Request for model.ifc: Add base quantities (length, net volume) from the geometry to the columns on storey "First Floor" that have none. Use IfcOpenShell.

First a look at what the model holds.

```python
import ifcopenshell
import ifcopenshell.util.element
import ifcopenshell.util.unit

model = ifcopenshell.open("model.ifc")
print(model.schema)
for unit_type in ("LENGTHUNIT", "AREAUNIT", "VOLUMEUNIT"):
    print(unit_type, ifcopenshell.util.unit.calculate_unit_scale(model, unit_type))
storey = next(s for s in model.by_type("IfcBuildingStorey") if s.Name == "First Floor")
columns = [e for e in ifcopenshell.util.element.get_decomposition(storey) if e.is_a("IfcColumn")]
for e in sorted(columns, key=lambda e: e.id()):
    print(e.id(), e.is_a(), e.Name, list(ifcopenshell.util.element.get_psets(e, qtos_only=True)), sep=" | ")
```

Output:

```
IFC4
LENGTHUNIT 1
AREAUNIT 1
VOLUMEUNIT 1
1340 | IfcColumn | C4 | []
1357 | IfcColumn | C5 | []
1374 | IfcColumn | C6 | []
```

```python
import ifcopenshell
import ifcopenshell.api.pset
import ifcopenshell.geom
import ifcopenshell.util.element
import ifcopenshell.util.shape
import ifcopenshell.util.unit

model = ifcopenshell.open("model.ifc")
unit_scale = ifcopenshell.util.unit.calculate_unit_scale(model)
volume_scale = ifcopenshell.util.unit.calculate_unit_scale(model, "VOLUMEUNIT")
settings = ifcopenshell.geom.settings()

storey = next(s for s in model.by_type("IfcBuildingStorey") if s.Name == "First Floor")
columns = [e for e in ifcopenshell.util.element.get_decomposition(storey) if e.is_a("IfcColumn")]

for e in sorted(columns, key=lambda e: e.id()):
    if ifcopenshell.util.element.get_psets(e, qtos_only=True, should_inherit=False):
        continue
    # Geometry comes back in metres, in the element's own axes.
    shape = ifcopenshell.geom.create_shape(settings, e)
    values = {
        "Length": ifcopenshell.util.shape.get_z(shape.geometry) / unit_scale,
        "NetVolume": ifcopenshell.util.shape.get_volume(shape.geometry) / volume_scale,
    }
    qto = ifcopenshell.api.pset.add_qto(model, product=e, name="Qto_ColumnBaseQuantities")
    ifcopenshell.api.pset.edit_qto(model, qto=qto, properties=values)
    print(e.id(), {k: round(v, 3) for k, v in values.items()})

model.write("model_updated.ifc")
```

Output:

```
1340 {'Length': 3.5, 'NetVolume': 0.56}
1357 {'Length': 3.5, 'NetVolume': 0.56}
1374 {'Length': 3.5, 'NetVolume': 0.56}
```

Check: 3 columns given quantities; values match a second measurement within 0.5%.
